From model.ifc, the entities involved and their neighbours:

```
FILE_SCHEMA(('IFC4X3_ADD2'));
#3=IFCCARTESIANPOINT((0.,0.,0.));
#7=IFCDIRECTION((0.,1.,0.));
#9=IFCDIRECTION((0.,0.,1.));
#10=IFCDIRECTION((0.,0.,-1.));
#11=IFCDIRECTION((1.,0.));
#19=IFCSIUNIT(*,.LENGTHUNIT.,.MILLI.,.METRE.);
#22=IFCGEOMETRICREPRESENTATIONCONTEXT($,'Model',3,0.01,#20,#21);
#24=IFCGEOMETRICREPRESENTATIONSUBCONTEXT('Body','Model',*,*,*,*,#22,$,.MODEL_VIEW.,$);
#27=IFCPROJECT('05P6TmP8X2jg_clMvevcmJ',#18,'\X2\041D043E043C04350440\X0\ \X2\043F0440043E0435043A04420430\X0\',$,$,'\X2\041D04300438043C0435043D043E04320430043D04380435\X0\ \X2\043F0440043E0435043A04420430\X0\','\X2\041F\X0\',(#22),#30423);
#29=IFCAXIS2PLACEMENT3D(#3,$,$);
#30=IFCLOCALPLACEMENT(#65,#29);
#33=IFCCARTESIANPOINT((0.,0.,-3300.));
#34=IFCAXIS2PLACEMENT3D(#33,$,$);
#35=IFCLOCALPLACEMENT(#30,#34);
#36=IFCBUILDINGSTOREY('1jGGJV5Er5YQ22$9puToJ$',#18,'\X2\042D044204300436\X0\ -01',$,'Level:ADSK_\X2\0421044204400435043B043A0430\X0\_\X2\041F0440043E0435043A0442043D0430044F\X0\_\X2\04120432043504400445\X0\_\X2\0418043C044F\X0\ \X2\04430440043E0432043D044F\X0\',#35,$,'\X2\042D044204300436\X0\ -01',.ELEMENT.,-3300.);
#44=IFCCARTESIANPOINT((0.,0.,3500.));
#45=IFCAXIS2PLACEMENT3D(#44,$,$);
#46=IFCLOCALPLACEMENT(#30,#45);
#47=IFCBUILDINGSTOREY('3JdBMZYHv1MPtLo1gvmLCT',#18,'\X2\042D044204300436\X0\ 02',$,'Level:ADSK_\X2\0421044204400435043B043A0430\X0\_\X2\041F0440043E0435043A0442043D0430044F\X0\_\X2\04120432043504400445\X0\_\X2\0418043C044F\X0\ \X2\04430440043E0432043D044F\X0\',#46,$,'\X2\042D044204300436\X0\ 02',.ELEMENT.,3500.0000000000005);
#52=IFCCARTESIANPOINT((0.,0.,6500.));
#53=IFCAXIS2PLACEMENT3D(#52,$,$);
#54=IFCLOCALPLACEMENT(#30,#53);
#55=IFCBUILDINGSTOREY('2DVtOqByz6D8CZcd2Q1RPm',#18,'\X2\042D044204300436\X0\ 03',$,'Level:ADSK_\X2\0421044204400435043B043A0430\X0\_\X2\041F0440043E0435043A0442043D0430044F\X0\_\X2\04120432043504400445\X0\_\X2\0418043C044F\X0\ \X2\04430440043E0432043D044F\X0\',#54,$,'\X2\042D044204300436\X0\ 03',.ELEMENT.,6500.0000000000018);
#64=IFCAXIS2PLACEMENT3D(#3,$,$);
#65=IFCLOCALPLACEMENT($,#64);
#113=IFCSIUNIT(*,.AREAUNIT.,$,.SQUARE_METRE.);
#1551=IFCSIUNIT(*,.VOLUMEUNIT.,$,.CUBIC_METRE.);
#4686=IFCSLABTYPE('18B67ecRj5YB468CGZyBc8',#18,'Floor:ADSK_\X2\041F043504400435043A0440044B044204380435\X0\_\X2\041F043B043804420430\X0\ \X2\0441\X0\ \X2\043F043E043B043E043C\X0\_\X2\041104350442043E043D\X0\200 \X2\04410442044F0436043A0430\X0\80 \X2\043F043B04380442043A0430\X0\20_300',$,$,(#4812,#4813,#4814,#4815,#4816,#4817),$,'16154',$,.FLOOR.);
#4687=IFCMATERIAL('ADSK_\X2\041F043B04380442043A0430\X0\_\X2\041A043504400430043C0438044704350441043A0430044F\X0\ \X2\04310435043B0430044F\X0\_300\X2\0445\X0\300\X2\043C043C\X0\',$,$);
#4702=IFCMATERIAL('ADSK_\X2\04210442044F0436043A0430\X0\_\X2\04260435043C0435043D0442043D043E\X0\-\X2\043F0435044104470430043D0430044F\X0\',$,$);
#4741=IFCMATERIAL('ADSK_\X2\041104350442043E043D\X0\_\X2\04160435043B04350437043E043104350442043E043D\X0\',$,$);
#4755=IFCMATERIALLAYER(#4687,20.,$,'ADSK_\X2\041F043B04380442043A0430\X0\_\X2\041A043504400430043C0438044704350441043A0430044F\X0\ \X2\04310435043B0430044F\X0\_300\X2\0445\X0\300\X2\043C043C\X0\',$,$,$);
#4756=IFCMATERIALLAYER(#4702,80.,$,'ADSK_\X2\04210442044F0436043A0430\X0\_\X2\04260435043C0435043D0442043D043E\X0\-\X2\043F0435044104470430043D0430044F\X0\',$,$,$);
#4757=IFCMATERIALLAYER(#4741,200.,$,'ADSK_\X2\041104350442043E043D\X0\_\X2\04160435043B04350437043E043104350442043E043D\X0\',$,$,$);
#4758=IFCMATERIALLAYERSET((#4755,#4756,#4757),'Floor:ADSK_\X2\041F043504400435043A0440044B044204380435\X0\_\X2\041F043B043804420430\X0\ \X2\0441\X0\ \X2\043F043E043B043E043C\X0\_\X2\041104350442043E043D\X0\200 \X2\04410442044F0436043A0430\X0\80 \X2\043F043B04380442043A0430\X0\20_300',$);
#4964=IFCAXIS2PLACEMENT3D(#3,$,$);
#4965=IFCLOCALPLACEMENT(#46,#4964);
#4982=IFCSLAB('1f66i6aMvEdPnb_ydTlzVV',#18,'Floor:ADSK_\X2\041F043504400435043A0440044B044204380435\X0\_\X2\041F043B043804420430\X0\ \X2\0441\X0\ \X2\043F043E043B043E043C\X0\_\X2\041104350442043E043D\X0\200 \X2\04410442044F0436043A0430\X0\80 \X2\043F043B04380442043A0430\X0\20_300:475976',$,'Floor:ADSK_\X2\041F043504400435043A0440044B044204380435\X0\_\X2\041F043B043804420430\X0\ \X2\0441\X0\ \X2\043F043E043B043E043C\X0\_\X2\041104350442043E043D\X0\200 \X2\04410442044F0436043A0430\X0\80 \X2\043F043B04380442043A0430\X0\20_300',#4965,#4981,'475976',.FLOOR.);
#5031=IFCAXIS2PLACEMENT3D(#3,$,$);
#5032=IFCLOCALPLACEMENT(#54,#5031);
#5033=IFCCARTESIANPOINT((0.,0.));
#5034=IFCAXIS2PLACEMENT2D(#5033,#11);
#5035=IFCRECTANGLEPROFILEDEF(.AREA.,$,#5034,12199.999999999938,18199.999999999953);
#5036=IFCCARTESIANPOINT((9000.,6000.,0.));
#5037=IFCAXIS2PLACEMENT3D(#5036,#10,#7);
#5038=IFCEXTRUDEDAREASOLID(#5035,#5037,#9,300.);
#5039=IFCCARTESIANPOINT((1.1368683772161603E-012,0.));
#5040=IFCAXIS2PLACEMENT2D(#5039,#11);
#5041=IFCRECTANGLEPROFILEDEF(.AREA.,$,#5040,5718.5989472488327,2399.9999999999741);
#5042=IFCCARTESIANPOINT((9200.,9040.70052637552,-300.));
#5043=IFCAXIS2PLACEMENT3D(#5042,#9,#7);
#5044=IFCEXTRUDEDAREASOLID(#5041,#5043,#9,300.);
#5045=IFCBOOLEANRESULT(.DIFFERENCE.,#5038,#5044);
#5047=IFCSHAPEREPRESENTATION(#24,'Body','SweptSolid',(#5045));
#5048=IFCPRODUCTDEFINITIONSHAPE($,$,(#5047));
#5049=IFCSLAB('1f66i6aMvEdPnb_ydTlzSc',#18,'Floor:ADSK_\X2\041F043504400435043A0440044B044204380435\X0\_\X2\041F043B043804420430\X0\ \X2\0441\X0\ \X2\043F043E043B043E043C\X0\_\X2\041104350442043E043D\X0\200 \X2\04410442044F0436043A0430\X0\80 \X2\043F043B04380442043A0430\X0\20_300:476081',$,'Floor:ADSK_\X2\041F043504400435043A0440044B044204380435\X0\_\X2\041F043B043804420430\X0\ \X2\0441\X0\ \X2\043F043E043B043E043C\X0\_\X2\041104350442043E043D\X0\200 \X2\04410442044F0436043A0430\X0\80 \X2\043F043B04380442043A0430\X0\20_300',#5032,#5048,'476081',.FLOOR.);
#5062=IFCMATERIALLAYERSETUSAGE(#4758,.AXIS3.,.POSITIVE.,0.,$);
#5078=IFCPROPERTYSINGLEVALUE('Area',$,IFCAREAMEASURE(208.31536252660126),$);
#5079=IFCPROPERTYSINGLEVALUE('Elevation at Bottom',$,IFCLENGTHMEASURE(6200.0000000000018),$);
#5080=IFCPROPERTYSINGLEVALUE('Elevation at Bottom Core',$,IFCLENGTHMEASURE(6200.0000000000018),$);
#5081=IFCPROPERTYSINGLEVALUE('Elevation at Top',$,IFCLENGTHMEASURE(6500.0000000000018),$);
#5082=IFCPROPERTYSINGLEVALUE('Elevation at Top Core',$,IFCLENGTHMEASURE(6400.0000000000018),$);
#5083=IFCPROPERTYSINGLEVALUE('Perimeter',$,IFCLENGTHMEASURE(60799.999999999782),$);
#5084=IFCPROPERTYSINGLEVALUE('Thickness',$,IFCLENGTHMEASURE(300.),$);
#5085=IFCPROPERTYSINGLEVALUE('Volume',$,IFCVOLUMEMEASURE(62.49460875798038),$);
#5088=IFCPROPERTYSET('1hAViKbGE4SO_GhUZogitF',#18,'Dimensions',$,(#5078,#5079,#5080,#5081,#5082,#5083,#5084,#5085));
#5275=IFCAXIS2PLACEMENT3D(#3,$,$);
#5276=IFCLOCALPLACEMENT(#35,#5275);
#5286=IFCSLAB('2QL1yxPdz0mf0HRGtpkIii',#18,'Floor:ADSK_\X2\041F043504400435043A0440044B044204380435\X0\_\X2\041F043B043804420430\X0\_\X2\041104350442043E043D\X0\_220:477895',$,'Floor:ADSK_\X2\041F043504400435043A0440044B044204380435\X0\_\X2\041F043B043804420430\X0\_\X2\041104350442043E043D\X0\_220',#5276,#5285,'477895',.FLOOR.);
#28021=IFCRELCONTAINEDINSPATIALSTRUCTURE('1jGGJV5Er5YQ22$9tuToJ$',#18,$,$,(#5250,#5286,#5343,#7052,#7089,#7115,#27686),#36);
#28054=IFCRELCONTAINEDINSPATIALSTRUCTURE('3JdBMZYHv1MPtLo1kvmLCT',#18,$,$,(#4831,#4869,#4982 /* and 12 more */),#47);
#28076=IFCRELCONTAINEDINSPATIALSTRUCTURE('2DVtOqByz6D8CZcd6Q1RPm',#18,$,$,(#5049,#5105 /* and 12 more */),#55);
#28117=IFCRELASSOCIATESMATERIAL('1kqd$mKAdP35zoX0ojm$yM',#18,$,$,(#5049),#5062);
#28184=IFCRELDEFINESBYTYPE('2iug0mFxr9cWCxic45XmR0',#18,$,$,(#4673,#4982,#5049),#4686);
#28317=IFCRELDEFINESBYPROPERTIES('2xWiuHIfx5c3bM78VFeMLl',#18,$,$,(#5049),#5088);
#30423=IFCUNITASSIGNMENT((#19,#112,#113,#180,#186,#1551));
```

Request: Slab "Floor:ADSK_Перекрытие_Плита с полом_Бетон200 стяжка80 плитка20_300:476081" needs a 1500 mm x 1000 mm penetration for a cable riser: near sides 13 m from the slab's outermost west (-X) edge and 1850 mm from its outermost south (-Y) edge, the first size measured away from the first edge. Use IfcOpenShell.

```python
import numpy as np
import ifcopenshell
import ifcopenshell.api.feature
import ifcopenshell.api.geometry
import ifcopenshell.api.pset
import ifcopenshell.api.root
import ifcopenshell.geom
import ifcopenshell.util.element
import ifcopenshell.util.placement
import ifcopenshell.util.representation
import ifcopenshell.util.shape
import ifcopenshell.util.unit

model = ifcopenshell.open("model.ifc")
unit_scale = ifcopenshell.util.unit.calculate_unit_scale(model)
area_scale = ifcopenshell.util.unit.calculate_unit_scale(model, "AREAUNIT")
volume_scale = ifcopenshell.util.unit.calculate_unit_scale(model, "VOLUMEUNIT")
settings = ifcopenshell.geom.settings()


def volume(element):
    """Net volume in cubic metres, openings subtracted."""
    shape = ifcopenshell.geom.create_shape(settings, element)
    return ifcopenshell.util.shape.get_volume(shape.geometry)


slab = model.by_guid("1f66i6aMvEdPnb_ydTlzSc")
before = volume(slab)

# Extent in the slab's own axes, in metres. The edges named are its -X and -Y sides.
slab_shape = ifcopenshell.geom.create_shape(settings, slab)
vertices = ifcopenshell.util.shape.get_vertices(slab_shape.geometry)
x_min, y_min, bottom = vertices.min(axis=0)
top = vertices[:, 2].max()

opening = ifcopenshell.api.root.create_entity(model, ifc_class="IfcOpeningElement", name="Cable riser opening", predefined_type="OPENING")
context = ifcopenshell.util.representation.get_context(model, "Model", "Body", "MODEL_VIEW")
width, depth = 1.5, 1
outline = [(0.0, 0.0), (width, 0.0), (width, depth), (0.0, depth), (0.0, 0.0)]
# Overshoot both faces by 50 mm so the cut is clean.
shape = ifcopenshell.api.geometry.add_slab_representation(
    model, context=context, depth=top - bottom + 0.1, polyline=outline
)
ifcopenshell.api.geometry.assign_representation(model, product=opening, representation=shape)

matrix = ifcopenshell.util.placement.get_local_placement(slab.ObjectPlacement)
matrix[:, 3] = matrix @ np.append(np.array([x_min + 13, y_min + 1.85, bottom - 0.05]) / unit_scale, 1.0)
ifcopenshell.api.geometry.edit_object_placement(model, product=opening, matrix=matrix, is_si=False)
ifcopenshell.api.feature.add_feature(model, feature=opening, element=slab)

after = volume(slab)

# Update the slab's stored quantities.
pset = model.by_id(ifcopenshell.util.element.get_pset(slab, "Dimensions", should_inherit=False)["id"])
ifcopenshell.api.pset.edit_pset(model, pset=pset, properties={
    "Area": model.create_entity("IfcAreaMeasure", after / (top - bottom) / area_scale),
    "Volume": model.create_entity("IfcVolumeMeasure", after / volume_scale),
})

print(f"slab volume {before:.3f} -> {after:.3f} m3")

model.write("model_rev.ifc")
```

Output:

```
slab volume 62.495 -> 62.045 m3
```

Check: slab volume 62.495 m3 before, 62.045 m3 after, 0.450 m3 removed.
